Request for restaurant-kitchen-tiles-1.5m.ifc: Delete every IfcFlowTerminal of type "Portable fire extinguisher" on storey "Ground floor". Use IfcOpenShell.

First a look at what the model holds.

```python
import ifcopenshell
import ifcopenshell.util.element

model = ifcopenshell.open("restaurant-kitchen-tiles-1.5m.ifc")
print(model.schema)
storey = next(s for s in model.by_type("IfcBuildingStorey") if s.Name == "Ground floor")
terminals = [e for e in ifcopenshell.util.element.get_decomposition(storey) if e.is_a("IfcFlowTerminal")]
seen = {}
for e in terminals:
    element_type = ifcopenshell.util.element.get_type(e)
    name = element_type.Name if element_type not in (None, e) else None
    seen[name] = seen.get(name, 0) + 1
for name, count in sorted(seen.items(), key=str):
    print(count, "x", name)
```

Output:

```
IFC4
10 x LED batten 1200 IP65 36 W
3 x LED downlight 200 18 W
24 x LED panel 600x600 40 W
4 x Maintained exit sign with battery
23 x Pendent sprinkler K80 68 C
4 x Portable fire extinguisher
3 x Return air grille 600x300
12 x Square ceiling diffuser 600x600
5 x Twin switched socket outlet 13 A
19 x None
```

```python
import ifcopenshell
import ifcopenshell.api.root
import ifcopenshell.util.element

model = ifcopenshell.open("restaurant-kitchen-tiles-1.5m.ifc")

storey = next(s for s in model.by_type("IfcBuildingStorey") if s.Name == "Ground floor")
terminals = [e for e in ifcopenshell.util.element.get_decomposition(storey) if e.is_a("IfcFlowTerminal")]
targets = [e for e in terminals if (t := ifcopenshell.util.element.get_type(e)) not in (None, e) and t.Name == "Portable fire extinguisher"]

for e in targets:
    ifcopenshell.api.root.remove_product(model, product=e)
print(len(targets), "removed")

model.write("restaurant-kitchen-tiles-1.5m_edited.ifc")
```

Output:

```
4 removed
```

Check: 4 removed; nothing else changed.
